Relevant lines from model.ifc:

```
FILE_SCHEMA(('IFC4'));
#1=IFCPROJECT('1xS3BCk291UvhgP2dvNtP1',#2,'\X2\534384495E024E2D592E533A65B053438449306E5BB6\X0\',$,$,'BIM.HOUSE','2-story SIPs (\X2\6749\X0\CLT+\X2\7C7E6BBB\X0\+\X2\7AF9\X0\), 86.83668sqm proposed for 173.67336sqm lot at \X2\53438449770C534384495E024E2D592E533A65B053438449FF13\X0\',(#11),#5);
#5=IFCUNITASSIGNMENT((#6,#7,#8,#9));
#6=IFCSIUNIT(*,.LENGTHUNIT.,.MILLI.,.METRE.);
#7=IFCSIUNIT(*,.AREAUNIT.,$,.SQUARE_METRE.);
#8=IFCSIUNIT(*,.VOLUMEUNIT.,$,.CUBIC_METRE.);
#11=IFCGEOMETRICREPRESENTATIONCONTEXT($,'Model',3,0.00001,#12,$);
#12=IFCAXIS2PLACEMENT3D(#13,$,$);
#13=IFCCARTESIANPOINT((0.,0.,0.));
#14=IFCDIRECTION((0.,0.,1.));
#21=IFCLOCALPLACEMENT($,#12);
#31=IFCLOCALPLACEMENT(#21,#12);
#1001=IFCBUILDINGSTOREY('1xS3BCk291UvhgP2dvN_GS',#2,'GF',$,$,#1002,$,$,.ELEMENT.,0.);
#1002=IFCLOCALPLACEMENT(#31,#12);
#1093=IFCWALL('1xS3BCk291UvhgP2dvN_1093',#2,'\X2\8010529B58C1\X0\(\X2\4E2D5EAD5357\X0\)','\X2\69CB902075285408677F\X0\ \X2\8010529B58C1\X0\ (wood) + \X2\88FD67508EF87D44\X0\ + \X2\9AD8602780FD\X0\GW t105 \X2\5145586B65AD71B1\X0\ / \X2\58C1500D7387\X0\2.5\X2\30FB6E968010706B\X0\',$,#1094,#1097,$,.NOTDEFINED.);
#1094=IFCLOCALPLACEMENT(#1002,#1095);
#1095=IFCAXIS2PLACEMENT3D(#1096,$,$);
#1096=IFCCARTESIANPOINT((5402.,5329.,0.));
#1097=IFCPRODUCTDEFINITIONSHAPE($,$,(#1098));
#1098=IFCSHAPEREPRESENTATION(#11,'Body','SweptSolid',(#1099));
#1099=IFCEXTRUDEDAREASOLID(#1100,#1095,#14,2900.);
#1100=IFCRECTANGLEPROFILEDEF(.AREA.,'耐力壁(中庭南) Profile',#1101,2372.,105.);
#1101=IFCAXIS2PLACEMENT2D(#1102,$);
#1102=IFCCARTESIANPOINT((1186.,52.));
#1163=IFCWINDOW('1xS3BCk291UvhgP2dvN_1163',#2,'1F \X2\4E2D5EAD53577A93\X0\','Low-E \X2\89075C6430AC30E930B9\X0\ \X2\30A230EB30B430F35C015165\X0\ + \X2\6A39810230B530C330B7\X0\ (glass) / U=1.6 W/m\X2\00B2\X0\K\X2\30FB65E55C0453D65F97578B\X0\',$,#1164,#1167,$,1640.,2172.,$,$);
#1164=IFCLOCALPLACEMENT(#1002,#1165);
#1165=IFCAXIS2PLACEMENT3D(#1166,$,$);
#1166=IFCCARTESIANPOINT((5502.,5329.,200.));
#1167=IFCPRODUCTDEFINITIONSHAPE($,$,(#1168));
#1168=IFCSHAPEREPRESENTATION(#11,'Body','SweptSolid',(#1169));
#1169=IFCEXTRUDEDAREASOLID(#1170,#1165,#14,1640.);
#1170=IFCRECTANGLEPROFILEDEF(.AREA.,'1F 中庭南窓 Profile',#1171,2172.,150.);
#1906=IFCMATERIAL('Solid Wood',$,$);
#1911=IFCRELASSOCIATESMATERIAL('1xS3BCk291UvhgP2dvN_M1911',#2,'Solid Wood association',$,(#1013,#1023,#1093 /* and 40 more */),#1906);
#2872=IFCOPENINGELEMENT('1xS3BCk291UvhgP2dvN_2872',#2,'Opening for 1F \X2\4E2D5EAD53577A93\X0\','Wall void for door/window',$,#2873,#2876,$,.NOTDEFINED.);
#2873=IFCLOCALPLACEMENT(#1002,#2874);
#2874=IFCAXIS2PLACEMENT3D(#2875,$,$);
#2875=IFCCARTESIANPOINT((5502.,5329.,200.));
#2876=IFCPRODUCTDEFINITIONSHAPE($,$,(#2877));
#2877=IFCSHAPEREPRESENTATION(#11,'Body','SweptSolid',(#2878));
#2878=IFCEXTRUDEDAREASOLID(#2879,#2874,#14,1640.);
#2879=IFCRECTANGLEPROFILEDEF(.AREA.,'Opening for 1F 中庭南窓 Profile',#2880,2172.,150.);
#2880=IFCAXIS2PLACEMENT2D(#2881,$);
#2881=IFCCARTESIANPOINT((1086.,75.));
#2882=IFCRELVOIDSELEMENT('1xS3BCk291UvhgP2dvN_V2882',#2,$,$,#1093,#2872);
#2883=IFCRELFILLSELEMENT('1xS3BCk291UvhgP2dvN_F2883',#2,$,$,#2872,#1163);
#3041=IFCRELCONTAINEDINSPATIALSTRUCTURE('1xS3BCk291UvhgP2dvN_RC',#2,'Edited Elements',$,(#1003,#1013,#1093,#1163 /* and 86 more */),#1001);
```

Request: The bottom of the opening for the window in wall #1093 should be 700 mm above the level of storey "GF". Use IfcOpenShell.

```python
import numpy as np
import ifcopenshell
import ifcopenshell.api.geometry
import ifcopenshell.geom
import ifcopenshell.util.element
import ifcopenshell.util.placement
import ifcopenshell.util.shape
import ifcopenshell.util.unit

model = ifcopenshell.open("model.ifc")
unit_scale = ifcopenshell.util.unit.calculate_unit_scale(model)

window = model.by_guid("1xS3BCk291UvhgP2dvN_1163")
opening = window.FillsVoids[0].RelatingOpeningElement
storey = ifcopenshell.util.element.get_container(window, ifc_class="IfcBuildingStorey")
level = ifcopenshell.util.placement.get_local_placement(storey.ObjectPlacement)[2, 3]

# The opening's origin need not be at the sill, so measure its lowest point.
shape = ifcopenshell.geom.create_shape(ifcopenshell.geom.settings(), opening)
bottom = ifcopenshell.util.shape.get_shape_bottom_elevation(shape, shape.geometry) / unit_scale
dz = level + 0.7 / unit_scale - bottom

shift = np.array([0.0, 0.0, dz])
# The window is not placed relative to its opening, so move both.
for product in (opening, window):
    matrix = ifcopenshell.util.placement.get_local_placement(product.ObjectPlacement)
    matrix[:3, 3] += shift
    ifcopenshell.api.geometry.edit_object_placement(model, product=product, matrix=matrix, is_si=False)

print(f"moved by {dz * unit_scale:+.3f} m")

model.write("model-out.ifc")
```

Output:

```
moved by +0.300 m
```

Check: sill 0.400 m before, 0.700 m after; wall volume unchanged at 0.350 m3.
